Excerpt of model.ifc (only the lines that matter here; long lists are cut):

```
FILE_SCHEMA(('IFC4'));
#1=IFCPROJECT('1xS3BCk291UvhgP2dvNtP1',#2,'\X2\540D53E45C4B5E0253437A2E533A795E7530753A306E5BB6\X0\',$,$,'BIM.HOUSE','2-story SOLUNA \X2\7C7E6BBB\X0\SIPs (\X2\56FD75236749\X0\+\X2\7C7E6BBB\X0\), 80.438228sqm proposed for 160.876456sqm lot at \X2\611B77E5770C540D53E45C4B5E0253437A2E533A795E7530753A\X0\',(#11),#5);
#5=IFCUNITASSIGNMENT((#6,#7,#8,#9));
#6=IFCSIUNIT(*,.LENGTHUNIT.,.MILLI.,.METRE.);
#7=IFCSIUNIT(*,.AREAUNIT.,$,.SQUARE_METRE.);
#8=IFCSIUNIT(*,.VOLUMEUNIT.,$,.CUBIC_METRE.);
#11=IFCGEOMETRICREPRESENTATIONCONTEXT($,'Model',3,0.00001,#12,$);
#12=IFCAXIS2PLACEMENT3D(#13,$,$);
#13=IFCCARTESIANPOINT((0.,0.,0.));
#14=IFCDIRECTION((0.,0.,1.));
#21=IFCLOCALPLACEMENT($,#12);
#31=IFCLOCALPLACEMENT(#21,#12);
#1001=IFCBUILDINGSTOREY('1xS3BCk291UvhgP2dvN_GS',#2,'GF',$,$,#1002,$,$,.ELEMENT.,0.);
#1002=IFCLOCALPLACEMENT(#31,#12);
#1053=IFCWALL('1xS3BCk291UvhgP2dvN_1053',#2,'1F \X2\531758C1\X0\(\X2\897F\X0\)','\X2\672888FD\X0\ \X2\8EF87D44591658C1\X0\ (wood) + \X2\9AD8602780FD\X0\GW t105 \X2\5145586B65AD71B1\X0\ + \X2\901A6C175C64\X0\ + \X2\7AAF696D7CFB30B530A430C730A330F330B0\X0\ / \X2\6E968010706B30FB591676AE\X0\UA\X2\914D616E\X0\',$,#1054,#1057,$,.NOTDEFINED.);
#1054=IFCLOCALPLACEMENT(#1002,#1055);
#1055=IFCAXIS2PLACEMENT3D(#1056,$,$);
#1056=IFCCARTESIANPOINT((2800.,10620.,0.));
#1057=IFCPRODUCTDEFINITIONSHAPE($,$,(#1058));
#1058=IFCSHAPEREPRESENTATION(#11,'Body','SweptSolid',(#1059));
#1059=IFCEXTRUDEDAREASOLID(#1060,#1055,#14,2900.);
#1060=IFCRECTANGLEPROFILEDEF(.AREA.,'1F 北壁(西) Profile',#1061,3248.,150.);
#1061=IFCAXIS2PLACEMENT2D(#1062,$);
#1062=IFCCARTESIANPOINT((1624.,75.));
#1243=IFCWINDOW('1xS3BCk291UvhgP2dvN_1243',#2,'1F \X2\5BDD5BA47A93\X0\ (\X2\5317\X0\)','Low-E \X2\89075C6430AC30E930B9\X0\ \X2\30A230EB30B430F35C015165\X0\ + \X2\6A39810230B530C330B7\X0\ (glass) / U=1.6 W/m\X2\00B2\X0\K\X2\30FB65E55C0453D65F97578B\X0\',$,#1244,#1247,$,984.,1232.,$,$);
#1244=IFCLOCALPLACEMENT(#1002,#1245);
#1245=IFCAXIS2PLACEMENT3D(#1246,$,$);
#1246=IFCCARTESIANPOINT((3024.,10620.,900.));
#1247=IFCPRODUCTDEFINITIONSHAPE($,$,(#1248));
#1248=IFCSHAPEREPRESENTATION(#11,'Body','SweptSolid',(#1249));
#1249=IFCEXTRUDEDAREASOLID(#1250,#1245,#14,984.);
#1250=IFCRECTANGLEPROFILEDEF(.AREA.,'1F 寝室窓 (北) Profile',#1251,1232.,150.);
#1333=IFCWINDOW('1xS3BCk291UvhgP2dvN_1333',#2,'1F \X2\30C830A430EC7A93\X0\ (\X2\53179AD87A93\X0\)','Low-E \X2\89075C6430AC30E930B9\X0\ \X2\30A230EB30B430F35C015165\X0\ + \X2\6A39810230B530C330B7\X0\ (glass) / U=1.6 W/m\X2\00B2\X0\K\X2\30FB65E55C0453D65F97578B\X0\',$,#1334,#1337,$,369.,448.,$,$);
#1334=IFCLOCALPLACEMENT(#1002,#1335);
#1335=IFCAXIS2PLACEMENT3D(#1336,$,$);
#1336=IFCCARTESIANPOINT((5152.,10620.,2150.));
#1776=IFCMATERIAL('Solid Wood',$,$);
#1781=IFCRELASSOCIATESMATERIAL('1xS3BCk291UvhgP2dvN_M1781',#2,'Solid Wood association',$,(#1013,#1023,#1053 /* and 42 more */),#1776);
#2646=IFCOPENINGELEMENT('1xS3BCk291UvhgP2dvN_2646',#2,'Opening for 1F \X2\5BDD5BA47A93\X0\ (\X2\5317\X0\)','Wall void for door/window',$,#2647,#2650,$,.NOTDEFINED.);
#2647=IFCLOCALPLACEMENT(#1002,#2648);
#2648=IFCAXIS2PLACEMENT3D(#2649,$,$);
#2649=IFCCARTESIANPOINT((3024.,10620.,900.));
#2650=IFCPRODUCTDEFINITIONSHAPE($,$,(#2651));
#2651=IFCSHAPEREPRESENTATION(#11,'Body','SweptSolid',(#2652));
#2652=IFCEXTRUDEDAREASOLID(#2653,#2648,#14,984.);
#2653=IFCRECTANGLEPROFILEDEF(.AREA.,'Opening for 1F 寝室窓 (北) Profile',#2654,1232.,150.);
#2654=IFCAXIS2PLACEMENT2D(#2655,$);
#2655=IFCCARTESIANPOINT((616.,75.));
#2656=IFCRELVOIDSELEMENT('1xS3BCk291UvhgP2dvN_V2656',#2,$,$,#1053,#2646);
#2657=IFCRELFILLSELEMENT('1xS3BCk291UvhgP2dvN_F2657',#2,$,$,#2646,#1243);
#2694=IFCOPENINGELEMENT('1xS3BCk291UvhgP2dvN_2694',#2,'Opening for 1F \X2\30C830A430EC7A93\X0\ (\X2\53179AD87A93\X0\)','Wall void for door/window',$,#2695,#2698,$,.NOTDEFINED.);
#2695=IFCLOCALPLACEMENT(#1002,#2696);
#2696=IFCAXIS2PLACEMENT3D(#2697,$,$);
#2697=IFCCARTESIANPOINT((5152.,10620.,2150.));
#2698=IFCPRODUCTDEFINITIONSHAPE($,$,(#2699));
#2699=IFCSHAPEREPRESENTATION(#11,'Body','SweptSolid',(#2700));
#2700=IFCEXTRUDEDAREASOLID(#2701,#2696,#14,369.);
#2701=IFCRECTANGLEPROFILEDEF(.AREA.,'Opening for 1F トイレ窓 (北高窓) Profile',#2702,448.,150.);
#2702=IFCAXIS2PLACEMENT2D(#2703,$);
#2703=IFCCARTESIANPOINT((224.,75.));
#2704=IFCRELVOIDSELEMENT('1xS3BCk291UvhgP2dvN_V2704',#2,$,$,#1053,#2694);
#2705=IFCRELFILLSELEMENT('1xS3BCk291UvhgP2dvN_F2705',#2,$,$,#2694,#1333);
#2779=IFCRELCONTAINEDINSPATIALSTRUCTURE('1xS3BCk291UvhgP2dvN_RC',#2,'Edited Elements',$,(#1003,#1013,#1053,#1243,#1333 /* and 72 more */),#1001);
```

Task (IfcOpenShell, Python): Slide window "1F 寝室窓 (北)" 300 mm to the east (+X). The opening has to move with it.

```python
import ifcopenshell
import ifcopenshell.api.geometry
import ifcopenshell.util.placement

model = ifcopenshell.open("model.ifc")

window = model.by_guid("1xS3BCk291UvhgP2dvN_1243")
opening = window.FillsVoids[0].RelatingOpeningElement
wall = opening.VoidsElements[0].RelatingBuildingElement

wall_matrix = ifcopenshell.util.placement.get_local_placement(wall.ObjectPlacement)
shift = wall_matrix[:3, 0] * 300.0
before = ifcopenshell.util.placement.get_local_placement(window.ObjectPlacement)[:3, 3].copy()

# The window is not placed relative to its opening, so move both.
for product in (opening, window):
    matrix = ifcopenshell.util.placement.get_local_placement(product.ObjectPlacement)
    matrix[:3, 3] += shift
    ifcopenshell.api.geometry.edit_object_placement(model, product=product, matrix=matrix, is_si=False)

after = ifcopenshell.util.placement.get_local_placement(window.ObjectPlacement)[:3, 3]
print("window moved by", (after - before).round(3) + 0.0)

model.write("model-out.ifc")
```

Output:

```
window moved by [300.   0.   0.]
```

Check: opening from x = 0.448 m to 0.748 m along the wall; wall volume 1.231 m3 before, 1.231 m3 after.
